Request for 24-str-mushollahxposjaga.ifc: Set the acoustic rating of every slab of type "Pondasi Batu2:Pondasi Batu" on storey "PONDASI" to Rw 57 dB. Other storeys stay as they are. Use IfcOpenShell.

First a look at what the model holds.

```python
import ifcopenshell
import ifcopenshell.util.element

model = ifcopenshell.open("24-str-mushollahxposjaga.ifc")
print(model.schema)
storey = next(s for s in model.by_type("IfcBuildingStorey") if s.Name == "PONDASI")
slabs = [e for e in ifcopenshell.util.element.get_decomposition(storey) if e.is_a("IfcSlab")]
seen = {}
for e in slabs:
    element_type = ifcopenshell.util.element.get_type(e)
    key = (element_type.Name if element_type != e and element_type else None, ifcopenshell.util.element.get_pset(e, "Pset_SlabCommon", "AcousticRating"))
    seen[key] = seen.get(key, 0) + 1
for (name, value), count in sorted(seen.items(), key=str):
    print(count, "x", name, "|", value)
```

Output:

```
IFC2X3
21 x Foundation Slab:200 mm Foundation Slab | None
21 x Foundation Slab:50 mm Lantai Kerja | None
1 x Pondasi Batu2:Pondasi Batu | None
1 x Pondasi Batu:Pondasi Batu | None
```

```python
import ifcopenshell
import ifcopenshell.api.pset
import ifcopenshell.util.element

model = ifcopenshell.open("24-str-mushollahxposjaga.ifc")

storey = next(s for s in model.by_type("IfcBuildingStorey") if s.Name == "PONDASI")
slabs = [e for e in ifcopenshell.util.element.get_decomposition(storey) if e.is_a("IfcSlab")]

count = 0
for e in slabs:
    element_type = ifcopenshell.util.element.get_type(e)
    if element_type in (None, e) or element_type.Name != "Pondasi Batu2:Pondasi Batu":
        continue
    # add_pset returns the element's existing set when there is one.
    pset = ifcopenshell.api.pset.add_pset(model, product=e, name="Pset_SlabCommon")
    ifcopenshell.api.pset.edit_pset(model, pset=pset, properties={"AcousticRating": "Rw 57 dB"})
    count += 1

print(count, "slabs updated")

model.write("24-str-mushollahxposjaga-out.ifc")
```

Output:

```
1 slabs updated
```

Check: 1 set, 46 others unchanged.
